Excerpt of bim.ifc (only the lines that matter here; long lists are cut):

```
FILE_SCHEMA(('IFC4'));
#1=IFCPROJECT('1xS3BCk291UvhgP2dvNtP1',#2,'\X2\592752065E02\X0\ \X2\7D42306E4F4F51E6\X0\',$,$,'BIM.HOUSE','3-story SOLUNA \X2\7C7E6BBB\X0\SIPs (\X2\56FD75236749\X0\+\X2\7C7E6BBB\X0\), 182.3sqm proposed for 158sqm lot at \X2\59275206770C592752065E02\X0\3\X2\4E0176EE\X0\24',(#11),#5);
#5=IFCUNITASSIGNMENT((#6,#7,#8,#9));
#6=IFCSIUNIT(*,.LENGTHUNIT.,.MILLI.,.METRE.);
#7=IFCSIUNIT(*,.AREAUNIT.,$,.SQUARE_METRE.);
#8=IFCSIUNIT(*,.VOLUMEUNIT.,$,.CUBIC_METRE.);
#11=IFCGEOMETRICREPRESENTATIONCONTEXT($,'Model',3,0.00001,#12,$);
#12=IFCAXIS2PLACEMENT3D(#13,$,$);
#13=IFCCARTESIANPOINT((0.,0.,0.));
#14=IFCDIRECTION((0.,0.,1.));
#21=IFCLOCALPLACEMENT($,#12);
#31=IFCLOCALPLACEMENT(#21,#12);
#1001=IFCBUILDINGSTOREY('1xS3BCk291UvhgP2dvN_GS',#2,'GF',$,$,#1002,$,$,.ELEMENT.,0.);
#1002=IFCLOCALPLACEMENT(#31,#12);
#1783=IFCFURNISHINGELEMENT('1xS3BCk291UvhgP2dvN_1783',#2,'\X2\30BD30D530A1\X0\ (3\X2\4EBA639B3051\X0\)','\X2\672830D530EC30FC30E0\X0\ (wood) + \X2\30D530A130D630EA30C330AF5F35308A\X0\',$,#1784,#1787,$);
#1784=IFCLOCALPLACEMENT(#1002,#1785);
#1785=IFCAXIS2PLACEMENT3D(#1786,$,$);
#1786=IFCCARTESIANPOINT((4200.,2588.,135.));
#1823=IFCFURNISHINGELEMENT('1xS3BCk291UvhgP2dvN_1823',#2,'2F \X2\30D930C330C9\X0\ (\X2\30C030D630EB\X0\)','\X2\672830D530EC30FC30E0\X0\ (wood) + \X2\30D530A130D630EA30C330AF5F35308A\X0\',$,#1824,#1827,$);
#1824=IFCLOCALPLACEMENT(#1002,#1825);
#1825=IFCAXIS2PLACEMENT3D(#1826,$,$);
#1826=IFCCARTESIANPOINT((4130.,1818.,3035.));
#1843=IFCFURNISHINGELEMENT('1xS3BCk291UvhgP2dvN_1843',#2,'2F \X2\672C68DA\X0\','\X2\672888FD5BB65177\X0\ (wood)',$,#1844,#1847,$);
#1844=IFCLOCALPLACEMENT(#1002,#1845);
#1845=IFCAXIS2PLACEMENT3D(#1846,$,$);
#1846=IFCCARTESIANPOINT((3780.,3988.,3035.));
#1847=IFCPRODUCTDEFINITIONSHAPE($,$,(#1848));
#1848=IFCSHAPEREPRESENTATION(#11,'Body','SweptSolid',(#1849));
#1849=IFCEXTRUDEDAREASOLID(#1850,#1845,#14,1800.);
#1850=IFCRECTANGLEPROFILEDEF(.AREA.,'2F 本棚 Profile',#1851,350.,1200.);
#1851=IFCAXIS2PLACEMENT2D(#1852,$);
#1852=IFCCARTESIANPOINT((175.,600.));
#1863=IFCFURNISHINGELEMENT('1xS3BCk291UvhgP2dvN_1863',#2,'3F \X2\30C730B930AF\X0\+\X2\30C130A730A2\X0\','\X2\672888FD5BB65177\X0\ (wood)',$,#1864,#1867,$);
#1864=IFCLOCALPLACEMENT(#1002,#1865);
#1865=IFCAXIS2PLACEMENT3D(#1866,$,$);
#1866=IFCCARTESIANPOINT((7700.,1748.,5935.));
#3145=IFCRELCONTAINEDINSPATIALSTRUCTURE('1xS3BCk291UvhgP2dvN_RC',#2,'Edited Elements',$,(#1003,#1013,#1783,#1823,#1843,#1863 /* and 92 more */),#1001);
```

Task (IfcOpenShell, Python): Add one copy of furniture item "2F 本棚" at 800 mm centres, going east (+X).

```python
import numpy as np
import ifcopenshell
import ifcopenshell.api.geometry
import ifcopenshell.api.root
import ifcopenshell.util.element
import ifcopenshell.util.placement

model = ifcopenshell.open("bim.ifc")


def reuse_history(source, copy):
    """copy_class also copies each property set's owner history, people and application; keep the originals."""
    for rel in copy.IsDefinedBy:
        if rel.is_a("IfcRelDefinesByProperties") and (history := rel.RelatingPropertyDefinition.OwnerHistory):
            rel.RelatingPropertyDefinition.OwnerHistory = source.OwnerHistory
            ifcopenshell.util.element.remove_deep2(model, history)


source = model.by_guid("1xS3BCk291UvhgP2dvN_1843")
base = ifcopenshell.util.placement.get_local_placement(source.ObjectPlacement)
step = np.array([1.0, 0.0, 0.0]) * 800.0

for i in range(1, 2):
    copy = ifcopenshell.api.root.copy_class(model, product=source)
    copy.Representation = ifcopenshell.util.element.copy_deep(
        model, source.Representation, exclude=["IfcGeometricRepresentationContext", "IfcRepresentationMap"]
    )
    reuse_history(source, copy)
    matrix = base.copy()
    matrix[:3, 3] += i * step
    print("added at", matrix[:3, 3].round(3) + 0.0)
    ifcopenshell.api.geometry.edit_object_placement(model, product=copy, matrix=matrix, is_si=False)

model.write("bim_updated.ifc")
```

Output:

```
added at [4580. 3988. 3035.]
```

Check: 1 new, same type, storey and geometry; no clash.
